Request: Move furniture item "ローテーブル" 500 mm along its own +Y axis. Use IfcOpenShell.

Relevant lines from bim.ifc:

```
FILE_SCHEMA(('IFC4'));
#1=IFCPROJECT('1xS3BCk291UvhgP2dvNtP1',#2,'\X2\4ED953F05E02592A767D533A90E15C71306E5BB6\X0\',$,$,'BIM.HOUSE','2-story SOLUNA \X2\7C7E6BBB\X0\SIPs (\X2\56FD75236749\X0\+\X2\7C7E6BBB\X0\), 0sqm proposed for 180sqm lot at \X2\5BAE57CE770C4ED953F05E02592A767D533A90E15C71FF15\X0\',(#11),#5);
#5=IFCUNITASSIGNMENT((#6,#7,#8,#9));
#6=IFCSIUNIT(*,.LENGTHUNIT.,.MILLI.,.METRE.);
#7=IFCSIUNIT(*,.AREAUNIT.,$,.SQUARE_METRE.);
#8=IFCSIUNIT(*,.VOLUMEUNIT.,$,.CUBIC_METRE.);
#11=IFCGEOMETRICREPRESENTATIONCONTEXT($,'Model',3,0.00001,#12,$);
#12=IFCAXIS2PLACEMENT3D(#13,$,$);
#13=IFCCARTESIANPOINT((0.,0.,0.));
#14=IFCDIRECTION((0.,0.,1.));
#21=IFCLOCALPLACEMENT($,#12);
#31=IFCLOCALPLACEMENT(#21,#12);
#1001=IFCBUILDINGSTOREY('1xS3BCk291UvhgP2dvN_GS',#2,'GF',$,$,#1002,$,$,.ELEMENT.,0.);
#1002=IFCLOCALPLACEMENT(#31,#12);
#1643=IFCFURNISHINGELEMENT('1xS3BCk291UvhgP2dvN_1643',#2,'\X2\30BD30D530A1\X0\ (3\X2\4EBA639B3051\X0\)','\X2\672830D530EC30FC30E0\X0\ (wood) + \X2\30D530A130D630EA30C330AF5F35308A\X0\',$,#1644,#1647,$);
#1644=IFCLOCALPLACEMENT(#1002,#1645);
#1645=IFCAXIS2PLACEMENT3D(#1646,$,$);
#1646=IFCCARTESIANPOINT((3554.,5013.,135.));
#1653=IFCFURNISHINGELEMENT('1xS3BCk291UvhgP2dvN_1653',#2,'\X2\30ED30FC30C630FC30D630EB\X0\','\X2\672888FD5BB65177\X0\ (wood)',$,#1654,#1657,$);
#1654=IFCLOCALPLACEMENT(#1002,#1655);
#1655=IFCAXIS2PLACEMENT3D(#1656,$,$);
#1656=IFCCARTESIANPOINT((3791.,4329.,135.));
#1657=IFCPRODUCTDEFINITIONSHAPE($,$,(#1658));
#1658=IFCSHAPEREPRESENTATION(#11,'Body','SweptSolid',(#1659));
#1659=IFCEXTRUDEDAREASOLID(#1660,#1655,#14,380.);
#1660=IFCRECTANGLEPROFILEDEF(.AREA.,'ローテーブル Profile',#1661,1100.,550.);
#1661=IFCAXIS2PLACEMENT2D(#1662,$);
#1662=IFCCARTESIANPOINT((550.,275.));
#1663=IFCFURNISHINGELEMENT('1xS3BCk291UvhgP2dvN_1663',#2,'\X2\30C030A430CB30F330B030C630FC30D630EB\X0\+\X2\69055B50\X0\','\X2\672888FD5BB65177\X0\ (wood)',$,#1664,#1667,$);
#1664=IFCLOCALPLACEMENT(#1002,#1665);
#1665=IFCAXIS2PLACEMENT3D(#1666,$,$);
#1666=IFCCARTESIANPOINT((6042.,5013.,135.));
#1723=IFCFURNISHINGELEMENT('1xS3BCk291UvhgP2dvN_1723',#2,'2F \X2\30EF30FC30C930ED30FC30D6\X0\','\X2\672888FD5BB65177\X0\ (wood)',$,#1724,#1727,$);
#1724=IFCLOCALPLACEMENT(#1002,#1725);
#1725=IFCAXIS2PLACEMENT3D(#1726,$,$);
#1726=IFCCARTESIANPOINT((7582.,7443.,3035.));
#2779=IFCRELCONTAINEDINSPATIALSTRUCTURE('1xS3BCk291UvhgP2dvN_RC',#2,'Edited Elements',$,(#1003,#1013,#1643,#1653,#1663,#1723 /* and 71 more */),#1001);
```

```python
import ifcopenshell
import ifcopenshell.api.geometry
import ifcopenshell.util.placement
import ifcopenshell.util.unit

model = ifcopenshell.open("bim.ifc")
unit_scale = ifcopenshell.util.unit.calculate_unit_scale(model)

item = model.by_guid("1xS3BCk291UvhgP2dvN_1653")
matrix = ifcopenshell.util.placement.get_local_placement(item.ObjectPlacement)
matrix[:3, 3] += matrix[:3, 1] * 0.5 / unit_scale
ifcopenshell.api.geometry.edit_object_placement(model, product=item, matrix=matrix, is_si=False)

print(ifcopenshell.util.placement.get_local_placement(item.ObjectPlacement).round(3) + 0.0)

model.write("bim-out.ifc")
```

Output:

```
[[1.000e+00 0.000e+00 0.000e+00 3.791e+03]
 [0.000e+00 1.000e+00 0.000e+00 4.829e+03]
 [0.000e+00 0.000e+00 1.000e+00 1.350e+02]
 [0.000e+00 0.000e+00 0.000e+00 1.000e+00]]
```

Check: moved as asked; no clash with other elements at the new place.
